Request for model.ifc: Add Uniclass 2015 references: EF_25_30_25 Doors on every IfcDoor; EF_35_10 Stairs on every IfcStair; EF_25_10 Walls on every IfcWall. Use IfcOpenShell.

First a look at what the model holds.

```python
import ifcopenshell

model = ifcopenshell.open("model.ifc")
print(model.schema)
print("classifications:", [c.Name for c in model.by_type("IfcClassification")])
for ifc_class in ("IfcDoor", "IfcRoof", "IfcStair", "IfcWall", "IfcWindow"):
    print(ifc_class, len(model.by_type(ifc_class)))
```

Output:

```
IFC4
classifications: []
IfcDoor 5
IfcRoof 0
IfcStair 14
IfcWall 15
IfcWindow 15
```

```python
import ifcopenshell
import ifcopenshell.api.classification

model = ifcopenshell.open("model.ifc")

system = ifcopenshell.api.classification.add_classification(model, classification="Uniclass 2015")

codes = {
    "IfcDoor": ("EF_25_30_25", "Doors"),
    "IfcStair": ("EF_35_10", "Stairs"),
    "IfcWall": ("EF_25_10", "Walls"),
}
for ifc_class, (code, name) in codes.items():
    products = model.by_type(ifc_class)
    ifcopenshell.api.classification.add_reference(
        model, products=products, classification=system, identification=code, name=name
    )
    print(code, len(products))

model.write("model_v2.ifc")
```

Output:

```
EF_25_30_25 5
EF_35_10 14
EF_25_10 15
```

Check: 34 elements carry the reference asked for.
